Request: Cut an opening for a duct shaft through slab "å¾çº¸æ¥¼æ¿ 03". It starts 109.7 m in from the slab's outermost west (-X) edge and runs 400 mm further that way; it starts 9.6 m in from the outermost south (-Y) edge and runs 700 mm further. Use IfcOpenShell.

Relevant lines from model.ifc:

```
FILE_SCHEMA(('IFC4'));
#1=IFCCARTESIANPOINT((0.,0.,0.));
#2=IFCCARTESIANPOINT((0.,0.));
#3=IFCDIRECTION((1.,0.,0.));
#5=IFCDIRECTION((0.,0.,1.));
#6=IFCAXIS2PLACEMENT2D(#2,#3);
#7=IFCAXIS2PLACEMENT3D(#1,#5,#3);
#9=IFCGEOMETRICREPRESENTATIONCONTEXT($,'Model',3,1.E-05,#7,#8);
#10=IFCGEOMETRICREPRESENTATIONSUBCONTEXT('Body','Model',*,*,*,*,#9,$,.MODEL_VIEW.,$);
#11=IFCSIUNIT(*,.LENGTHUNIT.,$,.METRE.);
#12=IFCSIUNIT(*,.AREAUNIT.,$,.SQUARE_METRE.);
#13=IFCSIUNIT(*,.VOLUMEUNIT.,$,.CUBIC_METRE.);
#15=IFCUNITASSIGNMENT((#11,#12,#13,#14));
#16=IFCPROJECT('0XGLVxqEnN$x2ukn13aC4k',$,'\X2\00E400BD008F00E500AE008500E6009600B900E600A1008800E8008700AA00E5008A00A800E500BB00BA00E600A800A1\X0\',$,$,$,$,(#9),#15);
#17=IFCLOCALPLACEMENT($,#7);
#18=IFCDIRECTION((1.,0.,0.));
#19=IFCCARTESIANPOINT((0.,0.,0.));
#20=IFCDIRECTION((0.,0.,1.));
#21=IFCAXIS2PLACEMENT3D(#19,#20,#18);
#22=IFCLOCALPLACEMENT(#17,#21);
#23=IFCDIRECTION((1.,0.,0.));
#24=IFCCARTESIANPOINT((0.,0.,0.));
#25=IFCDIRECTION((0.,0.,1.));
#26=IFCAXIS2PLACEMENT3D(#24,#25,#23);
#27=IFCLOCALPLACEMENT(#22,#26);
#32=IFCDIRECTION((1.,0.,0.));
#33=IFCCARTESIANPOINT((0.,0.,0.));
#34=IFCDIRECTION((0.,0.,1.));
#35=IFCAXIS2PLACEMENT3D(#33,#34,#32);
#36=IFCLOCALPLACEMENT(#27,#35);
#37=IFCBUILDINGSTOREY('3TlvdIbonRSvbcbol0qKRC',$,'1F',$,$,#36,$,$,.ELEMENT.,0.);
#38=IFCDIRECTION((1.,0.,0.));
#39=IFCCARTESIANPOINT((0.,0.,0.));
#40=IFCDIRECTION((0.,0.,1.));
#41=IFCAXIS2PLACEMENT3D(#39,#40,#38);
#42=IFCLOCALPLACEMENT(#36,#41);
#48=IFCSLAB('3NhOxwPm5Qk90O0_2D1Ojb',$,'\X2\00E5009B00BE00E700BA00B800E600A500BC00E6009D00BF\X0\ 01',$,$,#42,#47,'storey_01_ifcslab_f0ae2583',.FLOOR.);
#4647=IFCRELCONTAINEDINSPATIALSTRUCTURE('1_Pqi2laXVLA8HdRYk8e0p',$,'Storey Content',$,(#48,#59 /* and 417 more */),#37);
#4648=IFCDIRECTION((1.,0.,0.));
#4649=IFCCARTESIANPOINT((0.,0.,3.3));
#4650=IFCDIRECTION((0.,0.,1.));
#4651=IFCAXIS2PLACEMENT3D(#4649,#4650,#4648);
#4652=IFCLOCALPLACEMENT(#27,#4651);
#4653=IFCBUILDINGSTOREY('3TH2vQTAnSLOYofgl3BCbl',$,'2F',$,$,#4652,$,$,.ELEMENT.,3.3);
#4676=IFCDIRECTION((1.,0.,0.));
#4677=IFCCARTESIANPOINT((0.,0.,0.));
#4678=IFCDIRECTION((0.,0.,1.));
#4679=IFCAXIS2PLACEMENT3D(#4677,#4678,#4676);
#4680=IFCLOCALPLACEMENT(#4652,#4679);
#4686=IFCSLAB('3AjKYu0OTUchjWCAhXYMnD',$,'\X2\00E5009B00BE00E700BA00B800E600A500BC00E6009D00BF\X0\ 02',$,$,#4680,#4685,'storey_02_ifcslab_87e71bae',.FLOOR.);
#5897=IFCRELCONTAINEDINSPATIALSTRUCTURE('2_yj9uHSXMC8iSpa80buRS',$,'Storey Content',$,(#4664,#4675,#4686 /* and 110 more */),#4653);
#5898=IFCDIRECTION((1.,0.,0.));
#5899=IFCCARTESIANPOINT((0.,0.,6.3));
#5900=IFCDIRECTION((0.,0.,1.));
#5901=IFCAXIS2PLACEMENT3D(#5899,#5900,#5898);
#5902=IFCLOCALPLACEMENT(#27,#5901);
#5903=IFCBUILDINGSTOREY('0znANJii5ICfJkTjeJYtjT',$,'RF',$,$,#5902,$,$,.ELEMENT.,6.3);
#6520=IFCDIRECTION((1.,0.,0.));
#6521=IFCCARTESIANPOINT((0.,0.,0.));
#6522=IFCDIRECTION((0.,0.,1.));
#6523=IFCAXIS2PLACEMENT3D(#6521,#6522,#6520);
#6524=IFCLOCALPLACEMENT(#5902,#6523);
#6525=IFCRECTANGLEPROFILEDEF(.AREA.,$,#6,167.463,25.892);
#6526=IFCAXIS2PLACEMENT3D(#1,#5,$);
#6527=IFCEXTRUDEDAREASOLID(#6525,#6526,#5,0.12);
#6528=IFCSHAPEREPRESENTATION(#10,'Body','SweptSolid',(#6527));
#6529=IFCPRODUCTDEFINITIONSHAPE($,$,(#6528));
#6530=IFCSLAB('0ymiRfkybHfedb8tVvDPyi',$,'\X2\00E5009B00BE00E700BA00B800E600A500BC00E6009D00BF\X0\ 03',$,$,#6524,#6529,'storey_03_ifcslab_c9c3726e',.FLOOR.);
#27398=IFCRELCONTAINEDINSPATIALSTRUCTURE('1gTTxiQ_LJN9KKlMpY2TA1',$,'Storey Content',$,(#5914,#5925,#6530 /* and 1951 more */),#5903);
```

```python
import numpy as np
import ifcopenshell
import ifcopenshell.api.feature
import ifcopenshell.api.geometry
import ifcopenshell.api.root
import ifcopenshell.geom
import ifcopenshell.util.placement
import ifcopenshell.util.representation
import ifcopenshell.util.shape
import ifcopenshell.util.unit

model = ifcopenshell.open("model.ifc")
unit_scale = ifcopenshell.util.unit.calculate_unit_scale(model)
settings = ifcopenshell.geom.settings()


def volume(element):
    """Net volume in cubic metres, openings subtracted."""
    shape = ifcopenshell.geom.create_shape(settings, element)
    return ifcopenshell.util.shape.get_volume(shape.geometry)


slab = model.by_guid("0ymiRfkybHfedb8tVvDPyi")
before = volume(slab)

# Extent in the slab's own axes, in metres. The edges named are its -X and -Y sides.
slab_shape = ifcopenshell.geom.create_shape(settings, slab)
vertices = ifcopenshell.util.shape.get_vertices(slab_shape.geometry)
x_min, y_min, bottom = vertices.min(axis=0)
top = vertices[:, 2].max()

opening = ifcopenshell.api.root.create_entity(model, ifc_class="IfcOpeningElement", name="Duct shaft opening", predefined_type="OPENING")
context = ifcopenshell.util.representation.get_context(model, "Model", "Body", "MODEL_VIEW")
width, depth = 0.4, 0.7
outline = [(0.0, 0.0), (width, 0.0), (width, depth), (0.0, depth), (0.0, 0.0)]
# Overshoot both faces by 50 mm so the cut is clean.
shape = ifcopenshell.api.geometry.add_slab_representation(
    model, context=context, depth=top - bottom + 0.1, polyline=outline
)
ifcopenshell.api.geometry.assign_representation(model, product=opening, representation=shape)

matrix = ifcopenshell.util.placement.get_local_placement(slab.ObjectPlacement)
matrix[:, 3] = matrix @ np.append(np.array([x_min + 109.7, y_min + 9.6, bottom - 0.05]) / unit_scale, 1.0)
ifcopenshell.api.geometry.edit_object_placement(model, product=opening, matrix=matrix, is_si=False)
ifcopenshell.api.feature.add_feature(model, feature=opening, element=slab)

after = volume(slab)

print(f"slab volume {before:.3f} -> {after:.3f} m3")

model.write("model_edited.ifc")
```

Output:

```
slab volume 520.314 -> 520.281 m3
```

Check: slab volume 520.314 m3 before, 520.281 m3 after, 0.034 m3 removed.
